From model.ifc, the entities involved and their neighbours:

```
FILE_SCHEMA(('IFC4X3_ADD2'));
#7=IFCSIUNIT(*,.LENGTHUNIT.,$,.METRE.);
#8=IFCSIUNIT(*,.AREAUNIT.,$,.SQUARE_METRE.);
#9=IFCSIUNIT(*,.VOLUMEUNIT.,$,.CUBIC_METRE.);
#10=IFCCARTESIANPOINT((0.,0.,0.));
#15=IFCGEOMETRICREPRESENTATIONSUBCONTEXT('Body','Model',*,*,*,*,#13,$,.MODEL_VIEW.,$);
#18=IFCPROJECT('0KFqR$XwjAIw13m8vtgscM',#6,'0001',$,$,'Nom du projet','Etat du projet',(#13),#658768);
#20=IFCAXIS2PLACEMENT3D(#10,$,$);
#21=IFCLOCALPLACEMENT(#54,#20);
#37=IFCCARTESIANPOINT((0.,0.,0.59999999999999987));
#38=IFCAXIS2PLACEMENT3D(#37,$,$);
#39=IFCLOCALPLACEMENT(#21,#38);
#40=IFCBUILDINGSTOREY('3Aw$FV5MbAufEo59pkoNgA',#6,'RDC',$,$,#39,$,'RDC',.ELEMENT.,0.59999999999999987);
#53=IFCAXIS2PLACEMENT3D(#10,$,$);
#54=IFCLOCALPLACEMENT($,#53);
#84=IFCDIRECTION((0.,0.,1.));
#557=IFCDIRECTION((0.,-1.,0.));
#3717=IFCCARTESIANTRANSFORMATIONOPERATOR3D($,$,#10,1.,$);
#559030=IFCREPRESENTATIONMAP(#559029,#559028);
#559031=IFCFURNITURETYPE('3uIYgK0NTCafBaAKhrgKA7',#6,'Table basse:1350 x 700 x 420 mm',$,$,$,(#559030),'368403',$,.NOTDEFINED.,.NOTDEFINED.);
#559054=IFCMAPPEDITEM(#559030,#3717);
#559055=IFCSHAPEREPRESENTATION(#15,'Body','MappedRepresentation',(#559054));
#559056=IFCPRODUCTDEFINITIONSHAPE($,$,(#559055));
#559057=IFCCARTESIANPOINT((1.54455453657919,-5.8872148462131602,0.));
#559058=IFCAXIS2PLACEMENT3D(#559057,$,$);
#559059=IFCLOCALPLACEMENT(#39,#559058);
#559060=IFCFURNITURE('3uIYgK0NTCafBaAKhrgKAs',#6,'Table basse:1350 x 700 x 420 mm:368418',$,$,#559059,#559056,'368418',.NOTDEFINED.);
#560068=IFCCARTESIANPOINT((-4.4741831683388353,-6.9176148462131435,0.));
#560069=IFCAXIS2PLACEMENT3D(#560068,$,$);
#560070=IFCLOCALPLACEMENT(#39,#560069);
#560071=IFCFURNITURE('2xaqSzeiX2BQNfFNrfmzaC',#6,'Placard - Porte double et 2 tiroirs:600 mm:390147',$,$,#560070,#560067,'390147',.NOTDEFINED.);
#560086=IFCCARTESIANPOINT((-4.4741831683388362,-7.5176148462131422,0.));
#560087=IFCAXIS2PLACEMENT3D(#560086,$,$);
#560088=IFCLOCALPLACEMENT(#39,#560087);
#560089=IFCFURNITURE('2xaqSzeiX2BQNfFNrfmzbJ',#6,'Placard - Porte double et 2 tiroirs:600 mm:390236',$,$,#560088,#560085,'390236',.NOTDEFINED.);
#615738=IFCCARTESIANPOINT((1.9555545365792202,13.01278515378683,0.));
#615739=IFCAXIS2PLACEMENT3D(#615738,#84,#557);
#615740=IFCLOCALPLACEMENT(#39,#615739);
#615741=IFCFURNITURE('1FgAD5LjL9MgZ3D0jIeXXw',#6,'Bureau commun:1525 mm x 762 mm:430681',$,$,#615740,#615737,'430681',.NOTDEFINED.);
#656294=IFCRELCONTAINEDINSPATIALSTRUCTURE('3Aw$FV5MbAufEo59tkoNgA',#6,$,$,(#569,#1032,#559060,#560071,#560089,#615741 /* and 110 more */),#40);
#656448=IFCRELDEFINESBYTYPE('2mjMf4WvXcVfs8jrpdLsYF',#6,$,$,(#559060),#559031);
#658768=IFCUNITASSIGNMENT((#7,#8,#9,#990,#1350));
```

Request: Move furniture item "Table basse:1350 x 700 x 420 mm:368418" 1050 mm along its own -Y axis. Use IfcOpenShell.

```python
import ifcopenshell
import ifcopenshell.api.geometry
import ifcopenshell.util.placement
import ifcopenshell.util.unit

model = ifcopenshell.open("model.ifc")
unit_scale = ifcopenshell.util.unit.calculate_unit_scale(model)

item = model.by_guid("3uIYgK0NTCafBaAKhrgKAs")
matrix = ifcopenshell.util.placement.get_local_placement(item.ObjectPlacement)
matrix[:3, 3] -= matrix[:3, 1] * 1.05 / unit_scale
ifcopenshell.api.geometry.edit_object_placement(model, product=item, matrix=matrix, is_si=False)

print(ifcopenshell.util.placement.get_local_placement(item.ObjectPlacement).round(3) + 0.0)

model.write("model_updated.ifc")
```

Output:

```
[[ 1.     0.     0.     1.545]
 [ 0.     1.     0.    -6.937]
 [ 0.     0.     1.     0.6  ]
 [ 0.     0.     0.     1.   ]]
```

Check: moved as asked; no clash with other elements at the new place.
